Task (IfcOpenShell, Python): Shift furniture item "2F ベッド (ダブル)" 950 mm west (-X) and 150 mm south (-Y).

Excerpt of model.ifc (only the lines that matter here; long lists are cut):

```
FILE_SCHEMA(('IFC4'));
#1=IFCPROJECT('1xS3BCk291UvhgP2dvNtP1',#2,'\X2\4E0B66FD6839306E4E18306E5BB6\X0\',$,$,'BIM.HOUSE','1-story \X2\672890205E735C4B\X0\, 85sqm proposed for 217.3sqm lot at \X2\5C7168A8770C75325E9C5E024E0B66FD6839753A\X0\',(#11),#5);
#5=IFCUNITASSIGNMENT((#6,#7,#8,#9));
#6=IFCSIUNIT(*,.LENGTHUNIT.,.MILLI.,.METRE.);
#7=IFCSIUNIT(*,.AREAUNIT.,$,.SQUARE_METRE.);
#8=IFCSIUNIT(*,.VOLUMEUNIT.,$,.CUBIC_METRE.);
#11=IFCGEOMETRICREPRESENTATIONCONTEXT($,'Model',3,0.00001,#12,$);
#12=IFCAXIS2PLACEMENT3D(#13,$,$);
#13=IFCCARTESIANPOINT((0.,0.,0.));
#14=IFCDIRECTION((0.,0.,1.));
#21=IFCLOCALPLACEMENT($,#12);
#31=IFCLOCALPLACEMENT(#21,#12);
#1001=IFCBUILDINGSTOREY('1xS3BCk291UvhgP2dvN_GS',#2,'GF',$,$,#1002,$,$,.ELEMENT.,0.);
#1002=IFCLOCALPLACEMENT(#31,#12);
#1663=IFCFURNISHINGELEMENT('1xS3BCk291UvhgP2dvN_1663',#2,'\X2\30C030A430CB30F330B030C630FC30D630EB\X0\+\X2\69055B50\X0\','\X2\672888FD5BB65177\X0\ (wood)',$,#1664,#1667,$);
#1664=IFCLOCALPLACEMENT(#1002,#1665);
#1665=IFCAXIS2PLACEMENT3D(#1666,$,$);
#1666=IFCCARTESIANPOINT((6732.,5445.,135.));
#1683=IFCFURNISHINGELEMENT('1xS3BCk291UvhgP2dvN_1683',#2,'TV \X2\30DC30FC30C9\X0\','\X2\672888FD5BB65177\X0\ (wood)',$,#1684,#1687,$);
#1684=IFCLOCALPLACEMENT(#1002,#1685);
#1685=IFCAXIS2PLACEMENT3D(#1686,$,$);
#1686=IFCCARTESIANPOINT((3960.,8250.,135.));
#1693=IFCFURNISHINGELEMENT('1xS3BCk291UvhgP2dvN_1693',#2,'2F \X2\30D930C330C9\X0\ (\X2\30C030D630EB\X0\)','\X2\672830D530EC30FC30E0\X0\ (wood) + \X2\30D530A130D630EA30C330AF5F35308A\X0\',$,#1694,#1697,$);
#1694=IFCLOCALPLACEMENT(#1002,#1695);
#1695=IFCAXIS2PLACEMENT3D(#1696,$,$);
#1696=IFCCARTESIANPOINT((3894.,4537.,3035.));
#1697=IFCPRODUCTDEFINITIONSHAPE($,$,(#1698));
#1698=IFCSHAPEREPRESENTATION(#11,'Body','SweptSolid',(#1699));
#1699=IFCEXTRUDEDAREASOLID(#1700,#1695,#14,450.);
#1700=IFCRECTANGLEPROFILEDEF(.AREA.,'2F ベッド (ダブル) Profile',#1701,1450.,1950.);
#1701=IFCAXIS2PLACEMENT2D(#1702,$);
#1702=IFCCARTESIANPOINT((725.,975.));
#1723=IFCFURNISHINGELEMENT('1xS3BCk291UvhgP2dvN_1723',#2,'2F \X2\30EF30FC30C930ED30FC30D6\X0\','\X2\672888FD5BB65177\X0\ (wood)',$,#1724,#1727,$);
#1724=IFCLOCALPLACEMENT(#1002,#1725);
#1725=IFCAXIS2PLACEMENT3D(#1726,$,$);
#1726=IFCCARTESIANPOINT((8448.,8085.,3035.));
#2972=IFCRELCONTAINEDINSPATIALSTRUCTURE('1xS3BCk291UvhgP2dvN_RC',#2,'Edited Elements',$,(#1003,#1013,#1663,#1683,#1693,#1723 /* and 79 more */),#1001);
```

```python
import ifcopenshell
import ifcopenshell.api.geometry
import ifcopenshell.util.placement
import ifcopenshell.util.unit

model = ifcopenshell.open("model.ifc")
unit_scale = ifcopenshell.util.unit.calculate_unit_scale(model)

item = model.by_guid("1xS3BCk291UvhgP2dvN_1693")
matrix = ifcopenshell.util.placement.get_local_placement(item.ObjectPlacement)
matrix[0, 3] -= 0.95 / unit_scale
matrix[1, 3] -= 0.15 / unit_scale
ifcopenshell.api.geometry.edit_object_placement(model, product=item, matrix=matrix, is_si=False)

print(ifcopenshell.util.placement.get_local_placement(item.ObjectPlacement).round(3) + 0.0)

model.write("model_v2.ifc")
```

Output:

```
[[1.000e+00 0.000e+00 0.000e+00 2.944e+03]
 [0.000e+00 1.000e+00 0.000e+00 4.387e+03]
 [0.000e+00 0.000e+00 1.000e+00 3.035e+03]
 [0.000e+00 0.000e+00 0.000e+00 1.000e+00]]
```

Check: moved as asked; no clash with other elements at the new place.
